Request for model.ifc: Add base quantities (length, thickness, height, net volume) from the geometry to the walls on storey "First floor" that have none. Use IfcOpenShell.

First a look at what the model holds.

```python
import ifcopenshell
import ifcopenshell.util.element
import ifcopenshell.util.unit

model = ifcopenshell.open("model.ifc")
print(model.schema)
for unit_type in ("LENGTHUNIT", "AREAUNIT", "VOLUMEUNIT"):
    print(unit_type, ifcopenshell.util.unit.calculate_unit_scale(model, unit_type))
storey = next(s for s in model.by_type("IfcBuildingStorey") if s.Name == "First floor")
walls = [e for e in ifcopenshell.util.element.get_decomposition(storey) if e.is_a("IfcWall")]
for e in sorted(walls, key=lambda e: e.id()):
    print(e.id(), e.is_a(), e.Name, list(ifcopenshell.util.element.get_psets(e, qtos_only=True)), sep=" | ")
```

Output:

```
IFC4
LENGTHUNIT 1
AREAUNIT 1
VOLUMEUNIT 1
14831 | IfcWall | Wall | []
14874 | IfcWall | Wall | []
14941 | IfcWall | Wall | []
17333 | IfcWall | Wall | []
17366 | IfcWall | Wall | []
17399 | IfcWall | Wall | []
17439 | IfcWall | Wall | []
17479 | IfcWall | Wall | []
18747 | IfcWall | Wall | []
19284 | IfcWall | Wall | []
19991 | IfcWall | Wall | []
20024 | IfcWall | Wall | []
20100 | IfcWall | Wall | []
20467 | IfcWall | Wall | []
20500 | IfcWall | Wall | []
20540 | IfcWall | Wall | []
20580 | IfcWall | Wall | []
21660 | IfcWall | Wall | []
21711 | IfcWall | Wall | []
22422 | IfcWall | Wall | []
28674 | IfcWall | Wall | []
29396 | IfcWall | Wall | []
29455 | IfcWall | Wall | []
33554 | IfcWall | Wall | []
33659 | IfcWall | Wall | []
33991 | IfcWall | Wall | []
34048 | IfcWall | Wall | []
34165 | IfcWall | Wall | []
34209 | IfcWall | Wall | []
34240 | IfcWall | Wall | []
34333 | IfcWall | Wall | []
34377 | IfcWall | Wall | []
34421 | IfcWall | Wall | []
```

```python
import ifcopenshell
import ifcopenshell.api.pset
import ifcopenshell.geom
import ifcopenshell.util.element
import ifcopenshell.util.shape
import ifcopenshell.util.unit

model = ifcopenshell.open("model.ifc")
unit_scale = ifcopenshell.util.unit.calculate_unit_scale(model)
volume_scale = ifcopenshell.util.unit.calculate_unit_scale(model, "VOLUMEUNIT")
settings = ifcopenshell.geom.settings()

storey = next(s for s in model.by_type("IfcBuildingStorey") if s.Name == "First floor")
walls = [e for e in ifcopenshell.util.element.get_decomposition(storey) if e.is_a("IfcWall")]

for e in sorted(walls, key=lambda e: e.id()):
    if ifcopenshell.util.element.get_psets(e, qtos_only=True, should_inherit=False):
        continue
    # Geometry comes back in metres, in the element's own axes.
    shape = ifcopenshell.geom.create_shape(settings, e)
    values = {
        "Length": ifcopenshell.util.shape.get_x(shape.geometry) / unit_scale,
        "Width": ifcopenshell.util.shape.get_y(shape.geometry) / unit_scale,
        "Height": ifcopenshell.util.shape.get_z(shape.geometry) / unit_scale,
        "NetVolume": ifcopenshell.util.shape.get_volume(shape.geometry) / volume_scale,
    }
    qto = ifcopenshell.api.pset.add_qto(model, product=e, name="Qto_WallBaseQuantities")
    ifcopenshell.api.pset.edit_qto(model, qto=qto, properties=values)
    print(e.id(), {k: round(v, 3) for k, v in values.items()})

model.write("model_v2.ifc")
```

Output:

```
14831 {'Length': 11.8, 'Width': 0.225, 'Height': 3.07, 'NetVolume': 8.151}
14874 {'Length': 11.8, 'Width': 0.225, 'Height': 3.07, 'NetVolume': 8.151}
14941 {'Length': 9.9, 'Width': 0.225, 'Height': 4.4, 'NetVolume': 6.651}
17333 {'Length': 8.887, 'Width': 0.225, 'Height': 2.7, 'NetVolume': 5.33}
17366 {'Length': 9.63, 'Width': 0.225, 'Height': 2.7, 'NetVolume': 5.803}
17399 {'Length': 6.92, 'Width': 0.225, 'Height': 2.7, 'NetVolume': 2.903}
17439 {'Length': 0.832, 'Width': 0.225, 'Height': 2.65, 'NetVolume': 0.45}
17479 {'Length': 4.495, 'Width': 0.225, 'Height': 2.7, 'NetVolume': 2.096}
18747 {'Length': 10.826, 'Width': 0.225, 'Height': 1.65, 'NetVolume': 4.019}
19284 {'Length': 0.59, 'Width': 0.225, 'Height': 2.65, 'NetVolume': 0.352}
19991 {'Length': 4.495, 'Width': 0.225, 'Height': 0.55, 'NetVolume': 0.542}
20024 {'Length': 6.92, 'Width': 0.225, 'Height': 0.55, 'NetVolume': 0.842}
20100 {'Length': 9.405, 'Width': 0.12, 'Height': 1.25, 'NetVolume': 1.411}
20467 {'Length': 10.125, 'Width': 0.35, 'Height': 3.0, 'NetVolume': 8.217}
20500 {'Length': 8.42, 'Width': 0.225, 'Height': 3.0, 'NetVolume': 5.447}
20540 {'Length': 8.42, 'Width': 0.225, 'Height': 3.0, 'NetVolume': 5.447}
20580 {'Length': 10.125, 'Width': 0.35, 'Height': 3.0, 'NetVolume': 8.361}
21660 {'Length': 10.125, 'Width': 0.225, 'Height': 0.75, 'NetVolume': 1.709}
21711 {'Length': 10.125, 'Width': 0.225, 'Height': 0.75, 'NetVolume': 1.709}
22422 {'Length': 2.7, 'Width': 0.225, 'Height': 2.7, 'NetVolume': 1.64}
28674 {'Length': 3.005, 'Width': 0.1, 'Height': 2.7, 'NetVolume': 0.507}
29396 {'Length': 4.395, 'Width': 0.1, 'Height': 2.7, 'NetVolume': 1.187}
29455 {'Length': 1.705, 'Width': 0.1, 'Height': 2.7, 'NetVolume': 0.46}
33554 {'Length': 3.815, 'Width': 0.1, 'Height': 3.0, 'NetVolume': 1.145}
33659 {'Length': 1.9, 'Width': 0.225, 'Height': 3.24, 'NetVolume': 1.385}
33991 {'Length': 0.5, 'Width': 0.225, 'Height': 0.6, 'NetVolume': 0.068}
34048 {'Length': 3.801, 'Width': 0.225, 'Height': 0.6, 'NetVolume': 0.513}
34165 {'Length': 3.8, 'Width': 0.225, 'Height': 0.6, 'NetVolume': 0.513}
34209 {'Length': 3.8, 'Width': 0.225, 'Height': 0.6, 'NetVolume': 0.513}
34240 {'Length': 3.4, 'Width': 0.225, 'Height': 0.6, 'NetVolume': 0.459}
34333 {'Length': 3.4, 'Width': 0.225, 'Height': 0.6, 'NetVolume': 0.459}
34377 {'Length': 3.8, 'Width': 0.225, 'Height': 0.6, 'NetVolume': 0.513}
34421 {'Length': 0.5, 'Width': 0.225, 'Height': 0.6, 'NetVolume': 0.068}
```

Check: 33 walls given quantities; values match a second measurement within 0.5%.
